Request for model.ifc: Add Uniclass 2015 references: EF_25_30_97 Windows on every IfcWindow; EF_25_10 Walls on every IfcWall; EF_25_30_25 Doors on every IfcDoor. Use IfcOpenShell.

First a look at what the model holds.

```python
import ifcopenshell

model = ifcopenshell.open("model.ifc")
print(model.schema)
print("classifications:", [c.Name for c in model.by_type("IfcClassification")])
for ifc_class in ("IfcDoor", "IfcRoof", "IfcStair", "IfcWall", "IfcWindow"):
    print(ifc_class, len(model.by_type(ifc_class)))
```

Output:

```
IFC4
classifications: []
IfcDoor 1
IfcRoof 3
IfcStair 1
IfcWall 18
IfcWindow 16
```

```python
import ifcopenshell
import ifcopenshell.api.classification

model = ifcopenshell.open("model.ifc")

system = ifcopenshell.api.classification.add_classification(model, classification="Uniclass 2015")

codes = {
    "IfcWindow": ("EF_25_30_97", "Windows"),
    "IfcWall": ("EF_25_10", "Walls"),
    "IfcDoor": ("EF_25_30_25", "Doors"),
}
for ifc_class, (code, name) in codes.items():
    products = model.by_type(ifc_class)
    ifcopenshell.api.classification.add_reference(
        model, products=products, classification=system, identification=code, name=name
    )
    print(code, len(products))

model.write("model-out.ifc")
```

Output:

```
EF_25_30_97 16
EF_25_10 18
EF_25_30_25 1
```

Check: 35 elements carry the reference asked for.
